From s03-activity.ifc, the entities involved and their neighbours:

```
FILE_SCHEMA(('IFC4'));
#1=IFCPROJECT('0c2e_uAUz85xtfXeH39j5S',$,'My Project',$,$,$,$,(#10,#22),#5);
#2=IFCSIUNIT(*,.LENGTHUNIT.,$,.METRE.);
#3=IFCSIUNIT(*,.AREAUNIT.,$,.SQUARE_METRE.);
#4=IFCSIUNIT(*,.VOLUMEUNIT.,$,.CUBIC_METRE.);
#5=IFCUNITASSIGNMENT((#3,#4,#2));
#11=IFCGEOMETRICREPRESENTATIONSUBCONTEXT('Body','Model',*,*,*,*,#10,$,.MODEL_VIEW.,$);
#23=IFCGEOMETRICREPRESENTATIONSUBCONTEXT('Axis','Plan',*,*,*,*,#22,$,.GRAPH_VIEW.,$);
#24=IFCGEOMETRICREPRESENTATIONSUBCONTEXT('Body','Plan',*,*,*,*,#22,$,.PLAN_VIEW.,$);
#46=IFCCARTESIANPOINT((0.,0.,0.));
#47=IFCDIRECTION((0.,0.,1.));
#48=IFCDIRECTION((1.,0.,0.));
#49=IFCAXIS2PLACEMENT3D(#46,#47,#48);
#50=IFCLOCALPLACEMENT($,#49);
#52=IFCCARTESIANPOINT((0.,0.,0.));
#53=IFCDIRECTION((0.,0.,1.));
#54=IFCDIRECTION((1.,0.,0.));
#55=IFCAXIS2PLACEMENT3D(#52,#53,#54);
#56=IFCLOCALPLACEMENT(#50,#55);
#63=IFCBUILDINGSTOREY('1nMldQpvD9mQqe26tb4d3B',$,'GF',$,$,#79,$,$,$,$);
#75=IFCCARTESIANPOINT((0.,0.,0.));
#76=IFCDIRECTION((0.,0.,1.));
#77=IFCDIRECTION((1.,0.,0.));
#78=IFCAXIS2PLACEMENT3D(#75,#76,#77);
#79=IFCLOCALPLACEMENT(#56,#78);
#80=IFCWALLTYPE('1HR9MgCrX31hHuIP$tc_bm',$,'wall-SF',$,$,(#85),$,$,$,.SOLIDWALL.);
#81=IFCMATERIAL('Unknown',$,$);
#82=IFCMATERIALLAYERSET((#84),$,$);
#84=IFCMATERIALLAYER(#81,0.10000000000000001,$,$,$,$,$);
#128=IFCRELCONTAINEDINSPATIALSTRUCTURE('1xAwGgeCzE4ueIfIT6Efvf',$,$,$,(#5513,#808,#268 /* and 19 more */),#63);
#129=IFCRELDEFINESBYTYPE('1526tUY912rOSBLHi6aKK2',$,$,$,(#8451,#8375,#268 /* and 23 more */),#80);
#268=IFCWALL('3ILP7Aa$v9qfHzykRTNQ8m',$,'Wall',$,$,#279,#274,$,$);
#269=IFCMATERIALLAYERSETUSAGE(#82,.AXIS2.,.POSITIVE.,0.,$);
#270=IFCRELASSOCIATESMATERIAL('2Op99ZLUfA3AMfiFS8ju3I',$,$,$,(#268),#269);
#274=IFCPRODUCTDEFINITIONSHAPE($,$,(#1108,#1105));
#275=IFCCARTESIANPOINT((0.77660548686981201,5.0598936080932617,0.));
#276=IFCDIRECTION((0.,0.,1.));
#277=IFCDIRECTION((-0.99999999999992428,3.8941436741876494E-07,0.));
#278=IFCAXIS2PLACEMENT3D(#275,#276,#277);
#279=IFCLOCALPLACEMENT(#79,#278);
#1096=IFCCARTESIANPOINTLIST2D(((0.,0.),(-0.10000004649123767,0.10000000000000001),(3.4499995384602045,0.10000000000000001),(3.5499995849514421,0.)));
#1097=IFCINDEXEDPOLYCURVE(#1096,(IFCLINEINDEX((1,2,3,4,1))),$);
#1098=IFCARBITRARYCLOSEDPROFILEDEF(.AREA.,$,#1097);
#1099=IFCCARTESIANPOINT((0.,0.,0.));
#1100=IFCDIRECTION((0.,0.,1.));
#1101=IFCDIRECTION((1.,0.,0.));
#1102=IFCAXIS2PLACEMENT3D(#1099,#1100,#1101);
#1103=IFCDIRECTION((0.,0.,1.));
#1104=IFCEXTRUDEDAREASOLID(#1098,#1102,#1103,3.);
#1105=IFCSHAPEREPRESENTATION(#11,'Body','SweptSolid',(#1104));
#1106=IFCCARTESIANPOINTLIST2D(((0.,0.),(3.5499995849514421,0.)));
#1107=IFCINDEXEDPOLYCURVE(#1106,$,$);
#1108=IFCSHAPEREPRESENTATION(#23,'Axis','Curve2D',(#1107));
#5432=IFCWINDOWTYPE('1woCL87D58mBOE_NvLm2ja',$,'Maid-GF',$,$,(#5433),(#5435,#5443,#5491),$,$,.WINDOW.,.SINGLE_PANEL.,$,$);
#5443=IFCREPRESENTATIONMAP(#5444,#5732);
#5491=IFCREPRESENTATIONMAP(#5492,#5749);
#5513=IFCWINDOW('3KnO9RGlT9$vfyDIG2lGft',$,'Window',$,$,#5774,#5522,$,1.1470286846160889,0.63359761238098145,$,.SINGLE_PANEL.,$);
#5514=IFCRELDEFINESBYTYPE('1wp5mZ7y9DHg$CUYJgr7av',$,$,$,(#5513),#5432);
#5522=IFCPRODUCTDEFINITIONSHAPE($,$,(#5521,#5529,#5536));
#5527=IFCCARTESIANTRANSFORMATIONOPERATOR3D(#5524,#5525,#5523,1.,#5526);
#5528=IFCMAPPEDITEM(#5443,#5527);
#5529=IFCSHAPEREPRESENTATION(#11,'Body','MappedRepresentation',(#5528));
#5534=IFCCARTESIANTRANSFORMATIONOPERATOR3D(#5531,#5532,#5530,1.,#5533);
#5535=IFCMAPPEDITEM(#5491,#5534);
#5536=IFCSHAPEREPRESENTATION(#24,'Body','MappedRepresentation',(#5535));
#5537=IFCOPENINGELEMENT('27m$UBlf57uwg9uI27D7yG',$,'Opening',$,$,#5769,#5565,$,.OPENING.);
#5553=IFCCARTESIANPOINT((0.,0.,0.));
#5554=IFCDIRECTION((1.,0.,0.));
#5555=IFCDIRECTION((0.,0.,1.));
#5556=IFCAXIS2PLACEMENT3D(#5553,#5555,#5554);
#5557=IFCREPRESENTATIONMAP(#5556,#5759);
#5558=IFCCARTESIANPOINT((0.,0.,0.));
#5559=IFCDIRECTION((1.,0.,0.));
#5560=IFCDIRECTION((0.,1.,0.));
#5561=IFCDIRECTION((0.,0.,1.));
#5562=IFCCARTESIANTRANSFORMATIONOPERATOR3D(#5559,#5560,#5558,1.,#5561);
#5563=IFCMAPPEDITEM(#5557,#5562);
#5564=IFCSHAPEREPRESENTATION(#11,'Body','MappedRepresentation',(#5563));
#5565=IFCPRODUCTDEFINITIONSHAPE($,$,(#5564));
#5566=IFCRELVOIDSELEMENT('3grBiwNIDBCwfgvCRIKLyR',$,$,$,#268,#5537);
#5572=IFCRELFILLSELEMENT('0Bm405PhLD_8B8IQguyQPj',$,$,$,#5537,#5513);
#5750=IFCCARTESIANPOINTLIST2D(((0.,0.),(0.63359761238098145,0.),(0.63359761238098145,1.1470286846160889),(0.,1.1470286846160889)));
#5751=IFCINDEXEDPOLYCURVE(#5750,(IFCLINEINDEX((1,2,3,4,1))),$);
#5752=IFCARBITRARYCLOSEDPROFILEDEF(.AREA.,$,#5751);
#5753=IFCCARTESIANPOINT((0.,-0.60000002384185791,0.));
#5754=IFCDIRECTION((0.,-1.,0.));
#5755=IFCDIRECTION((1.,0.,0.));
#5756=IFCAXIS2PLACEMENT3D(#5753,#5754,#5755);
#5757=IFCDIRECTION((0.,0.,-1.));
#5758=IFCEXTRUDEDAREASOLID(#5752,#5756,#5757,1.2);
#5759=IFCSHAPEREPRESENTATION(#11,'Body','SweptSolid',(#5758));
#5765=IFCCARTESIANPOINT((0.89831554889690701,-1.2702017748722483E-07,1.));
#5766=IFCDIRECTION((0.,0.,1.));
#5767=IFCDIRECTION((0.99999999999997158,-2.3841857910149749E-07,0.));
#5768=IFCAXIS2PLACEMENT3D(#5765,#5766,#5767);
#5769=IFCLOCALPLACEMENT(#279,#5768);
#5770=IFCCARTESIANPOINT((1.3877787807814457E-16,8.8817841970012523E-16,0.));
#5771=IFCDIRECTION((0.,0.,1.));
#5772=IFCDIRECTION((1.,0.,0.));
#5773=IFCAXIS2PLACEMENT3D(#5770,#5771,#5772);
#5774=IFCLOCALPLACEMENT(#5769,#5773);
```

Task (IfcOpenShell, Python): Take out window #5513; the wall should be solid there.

```python
import ifcopenshell
import ifcopenshell.api.feature
import ifcopenshell.api.root
import ifcopenshell.geom
import ifcopenshell.util.shape

model = ifcopenshell.open("s03-activity.ifc")
settings = ifcopenshell.geom.settings()


def volume(element):
    """Net volume in cubic metres, openings subtracted."""
    shape = ifcopenshell.geom.create_shape(settings, element)
    return ifcopenshell.util.shape.get_volume(shape.geometry)


window = model.by_guid("3KnO9RGlT9$vfyDIG2lGft")
opening = window.FillsVoids[0].RelatingOpeningElement
wall = opening.VoidsElements[0].RelatingBuildingElement
before = volume(wall)

ifcopenshell.api.root.remove_product(model, product=window)
ifcopenshell.api.feature.remove_feature(model, feature=opening)

after = volume(wall)

print(f"wall volume {before:.3f} -> {after:.3f} m3")

model.write("s03-activity_v2.ifc")
```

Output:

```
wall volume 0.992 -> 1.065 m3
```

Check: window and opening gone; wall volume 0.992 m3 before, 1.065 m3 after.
